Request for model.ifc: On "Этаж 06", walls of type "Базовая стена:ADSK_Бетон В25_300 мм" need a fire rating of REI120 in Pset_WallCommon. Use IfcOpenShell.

First a look at what the model holds.

```python
import ifcopenshell
import ifcopenshell.util.element

model = ifcopenshell.open("model.ifc")
print(model.schema)
storey = next(s for s in model.by_type("IfcBuildingStorey") if s.Name == "Этаж 06")
walls = [e for e in ifcopenshell.util.element.get_decomposition(storey) if e.is_a("IfcWall")]
seen = {}
for e in walls:
    element_type = ifcopenshell.util.element.get_type(e)
    key = (element_type.Name if element_type != e and element_type else None, ifcopenshell.util.element.get_pset(e, "Pset_WallCommon", "FireRating"))
    seen[key] = seen.get(key, 0) + 1
for (name, value), count in sorted(seen.items(), key=str):
    print(count, "x", name, "|", value)
```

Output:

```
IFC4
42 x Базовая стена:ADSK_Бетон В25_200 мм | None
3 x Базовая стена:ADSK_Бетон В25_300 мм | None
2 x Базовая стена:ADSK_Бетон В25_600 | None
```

```python
import ifcopenshell
import ifcopenshell.api.pset
import ifcopenshell.util.element

model = ifcopenshell.open("model.ifc")

storey = next(s for s in model.by_type("IfcBuildingStorey") if s.Name == "Этаж 06")
walls = [e for e in ifcopenshell.util.element.get_decomposition(storey) if e.is_a("IfcWall")]

count = 0
for e in walls:
    element_type = ifcopenshell.util.element.get_type(e)
    if element_type in (None, e) or element_type.Name != "Базовая стена:ADSK_Бетон В25_300 мм":
        continue
    # add_pset returns the element's existing set when there is one.
    pset = ifcopenshell.api.pset.add_pset(model, product=e, name="Pset_WallCommon")
    ifcopenshell.api.pset.edit_pset(model, pset=pset, properties={"FireRating": "REI120"})
    count += 1

print(count, "walls updated")

model.write("model-out.ifc")
```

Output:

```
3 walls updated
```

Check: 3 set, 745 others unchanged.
